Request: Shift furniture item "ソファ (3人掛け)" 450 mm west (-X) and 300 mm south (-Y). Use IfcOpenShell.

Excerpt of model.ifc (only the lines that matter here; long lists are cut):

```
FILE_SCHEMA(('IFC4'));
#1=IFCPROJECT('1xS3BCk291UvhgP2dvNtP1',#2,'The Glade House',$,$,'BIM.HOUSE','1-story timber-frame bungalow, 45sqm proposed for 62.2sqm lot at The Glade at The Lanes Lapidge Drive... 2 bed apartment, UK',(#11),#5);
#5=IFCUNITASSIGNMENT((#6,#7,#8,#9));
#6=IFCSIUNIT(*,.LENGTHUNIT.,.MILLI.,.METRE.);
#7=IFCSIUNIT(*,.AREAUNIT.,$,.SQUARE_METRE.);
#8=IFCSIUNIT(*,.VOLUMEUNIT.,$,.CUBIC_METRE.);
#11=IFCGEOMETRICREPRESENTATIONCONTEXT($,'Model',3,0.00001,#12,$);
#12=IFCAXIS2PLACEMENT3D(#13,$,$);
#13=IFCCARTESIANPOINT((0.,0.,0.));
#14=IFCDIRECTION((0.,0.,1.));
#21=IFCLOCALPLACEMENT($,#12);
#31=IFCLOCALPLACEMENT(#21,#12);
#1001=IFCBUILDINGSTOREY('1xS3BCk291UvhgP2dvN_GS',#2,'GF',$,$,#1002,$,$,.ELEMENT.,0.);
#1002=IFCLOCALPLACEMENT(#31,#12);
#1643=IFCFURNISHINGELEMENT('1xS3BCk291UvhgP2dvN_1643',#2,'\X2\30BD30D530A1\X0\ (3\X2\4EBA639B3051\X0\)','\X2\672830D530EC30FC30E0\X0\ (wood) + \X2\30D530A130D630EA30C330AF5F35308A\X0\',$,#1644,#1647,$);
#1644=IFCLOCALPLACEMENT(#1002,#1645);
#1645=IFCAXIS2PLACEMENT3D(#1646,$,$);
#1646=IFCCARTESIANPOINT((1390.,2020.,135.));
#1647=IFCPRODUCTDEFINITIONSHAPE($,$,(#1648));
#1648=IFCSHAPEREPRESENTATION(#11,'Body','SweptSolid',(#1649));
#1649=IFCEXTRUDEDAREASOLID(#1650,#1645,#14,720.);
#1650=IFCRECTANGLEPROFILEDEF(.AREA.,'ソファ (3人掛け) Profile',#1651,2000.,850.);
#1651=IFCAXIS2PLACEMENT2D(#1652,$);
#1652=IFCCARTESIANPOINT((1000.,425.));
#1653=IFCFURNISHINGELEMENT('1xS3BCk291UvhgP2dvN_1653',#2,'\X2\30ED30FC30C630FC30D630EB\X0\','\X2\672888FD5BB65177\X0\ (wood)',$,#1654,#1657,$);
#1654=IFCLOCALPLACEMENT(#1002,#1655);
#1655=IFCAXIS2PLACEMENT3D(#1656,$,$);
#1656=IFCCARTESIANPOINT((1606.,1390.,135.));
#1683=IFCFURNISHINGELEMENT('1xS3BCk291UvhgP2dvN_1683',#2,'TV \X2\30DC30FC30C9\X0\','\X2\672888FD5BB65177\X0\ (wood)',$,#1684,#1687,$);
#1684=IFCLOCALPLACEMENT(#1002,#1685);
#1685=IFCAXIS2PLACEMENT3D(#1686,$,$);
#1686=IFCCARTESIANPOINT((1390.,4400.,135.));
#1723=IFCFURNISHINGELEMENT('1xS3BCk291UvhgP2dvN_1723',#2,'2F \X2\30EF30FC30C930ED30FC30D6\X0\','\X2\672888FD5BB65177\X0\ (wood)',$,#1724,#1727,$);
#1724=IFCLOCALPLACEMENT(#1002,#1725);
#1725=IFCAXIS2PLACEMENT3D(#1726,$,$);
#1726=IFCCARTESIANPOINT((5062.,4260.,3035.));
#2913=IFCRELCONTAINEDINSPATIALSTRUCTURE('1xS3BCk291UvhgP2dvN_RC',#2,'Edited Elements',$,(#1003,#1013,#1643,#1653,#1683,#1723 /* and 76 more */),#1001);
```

```python
import ifcopenshell
import ifcopenshell.api.geometry
import ifcopenshell.util.placement
import ifcopenshell.util.unit

model = ifcopenshell.open("model.ifc")
unit_scale = ifcopenshell.util.unit.calculate_unit_scale(model)

item = model.by_guid("1xS3BCk291UvhgP2dvN_1643")
matrix = ifcopenshell.util.placement.get_local_placement(item.ObjectPlacement)
matrix[0, 3] -= 0.45 / unit_scale
matrix[1, 3] -= 0.3 / unit_scale
ifcopenshell.api.geometry.edit_object_placement(model, product=item, matrix=matrix, is_si=False)

print(ifcopenshell.util.placement.get_local_placement(item.ObjectPlacement).round(3) + 0.0)

model.write("model_updated.ifc")
```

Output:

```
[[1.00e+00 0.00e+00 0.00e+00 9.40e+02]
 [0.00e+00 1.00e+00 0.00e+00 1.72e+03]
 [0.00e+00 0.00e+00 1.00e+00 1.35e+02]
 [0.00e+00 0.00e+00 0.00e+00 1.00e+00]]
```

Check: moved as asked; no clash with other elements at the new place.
